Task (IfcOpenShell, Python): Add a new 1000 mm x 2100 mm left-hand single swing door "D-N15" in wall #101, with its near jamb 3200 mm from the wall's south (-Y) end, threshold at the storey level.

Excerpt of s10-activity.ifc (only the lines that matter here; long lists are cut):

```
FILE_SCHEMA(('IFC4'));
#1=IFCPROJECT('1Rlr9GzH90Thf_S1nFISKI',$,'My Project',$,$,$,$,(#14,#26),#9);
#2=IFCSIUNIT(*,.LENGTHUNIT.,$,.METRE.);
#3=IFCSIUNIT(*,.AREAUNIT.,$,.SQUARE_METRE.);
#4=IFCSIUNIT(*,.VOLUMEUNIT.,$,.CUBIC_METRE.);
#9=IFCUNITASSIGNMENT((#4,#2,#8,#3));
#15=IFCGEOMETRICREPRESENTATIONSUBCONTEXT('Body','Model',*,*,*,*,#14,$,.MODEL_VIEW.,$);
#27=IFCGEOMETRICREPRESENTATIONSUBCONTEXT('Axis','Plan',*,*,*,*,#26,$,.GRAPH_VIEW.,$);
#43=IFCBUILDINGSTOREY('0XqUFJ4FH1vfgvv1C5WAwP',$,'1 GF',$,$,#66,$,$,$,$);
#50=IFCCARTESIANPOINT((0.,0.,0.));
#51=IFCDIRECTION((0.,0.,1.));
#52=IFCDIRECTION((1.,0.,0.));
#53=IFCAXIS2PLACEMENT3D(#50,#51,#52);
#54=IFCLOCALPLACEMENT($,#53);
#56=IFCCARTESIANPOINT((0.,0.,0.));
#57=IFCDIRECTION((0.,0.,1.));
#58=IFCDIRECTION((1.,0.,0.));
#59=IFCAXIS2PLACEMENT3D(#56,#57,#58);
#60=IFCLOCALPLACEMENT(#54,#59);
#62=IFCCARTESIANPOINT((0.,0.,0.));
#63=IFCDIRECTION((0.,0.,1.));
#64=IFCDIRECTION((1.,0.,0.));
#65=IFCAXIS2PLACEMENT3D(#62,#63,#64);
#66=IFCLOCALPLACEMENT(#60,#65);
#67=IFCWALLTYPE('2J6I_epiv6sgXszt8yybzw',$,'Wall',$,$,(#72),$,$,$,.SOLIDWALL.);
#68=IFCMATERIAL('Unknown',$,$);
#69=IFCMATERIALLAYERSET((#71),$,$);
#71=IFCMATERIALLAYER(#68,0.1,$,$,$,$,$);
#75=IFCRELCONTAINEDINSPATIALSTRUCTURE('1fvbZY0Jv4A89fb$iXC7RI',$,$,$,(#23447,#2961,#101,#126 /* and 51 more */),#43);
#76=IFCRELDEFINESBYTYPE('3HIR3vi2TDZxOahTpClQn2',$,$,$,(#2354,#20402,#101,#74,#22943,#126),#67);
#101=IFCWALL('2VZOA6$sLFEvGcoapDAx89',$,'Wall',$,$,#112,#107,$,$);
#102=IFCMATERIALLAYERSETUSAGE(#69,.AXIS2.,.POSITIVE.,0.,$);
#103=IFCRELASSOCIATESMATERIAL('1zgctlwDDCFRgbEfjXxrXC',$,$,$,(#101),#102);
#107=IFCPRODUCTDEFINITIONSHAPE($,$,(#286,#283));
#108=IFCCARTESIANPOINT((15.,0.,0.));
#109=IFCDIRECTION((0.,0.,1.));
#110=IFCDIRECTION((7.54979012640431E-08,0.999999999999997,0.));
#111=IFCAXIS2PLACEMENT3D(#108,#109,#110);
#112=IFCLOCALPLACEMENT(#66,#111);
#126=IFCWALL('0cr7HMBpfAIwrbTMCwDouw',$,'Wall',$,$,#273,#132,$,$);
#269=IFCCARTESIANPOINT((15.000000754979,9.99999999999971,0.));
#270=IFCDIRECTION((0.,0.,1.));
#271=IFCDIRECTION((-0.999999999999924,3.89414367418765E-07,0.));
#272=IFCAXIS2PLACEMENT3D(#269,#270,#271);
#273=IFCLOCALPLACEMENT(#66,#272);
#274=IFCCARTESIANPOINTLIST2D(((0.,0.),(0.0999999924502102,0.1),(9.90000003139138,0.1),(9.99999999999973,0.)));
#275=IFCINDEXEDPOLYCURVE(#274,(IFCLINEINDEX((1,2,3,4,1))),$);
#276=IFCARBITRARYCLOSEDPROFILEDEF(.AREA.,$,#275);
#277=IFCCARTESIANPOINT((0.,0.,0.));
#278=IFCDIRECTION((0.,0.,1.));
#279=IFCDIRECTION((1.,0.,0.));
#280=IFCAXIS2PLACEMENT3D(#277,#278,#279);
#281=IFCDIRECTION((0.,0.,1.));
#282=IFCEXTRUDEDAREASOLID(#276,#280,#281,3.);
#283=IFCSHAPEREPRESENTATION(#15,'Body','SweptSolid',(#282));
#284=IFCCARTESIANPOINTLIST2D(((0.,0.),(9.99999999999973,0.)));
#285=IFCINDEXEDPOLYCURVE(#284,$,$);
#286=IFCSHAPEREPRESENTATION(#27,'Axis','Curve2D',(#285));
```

```python
import numpy as np
import ifcopenshell
import ifcopenshell.api.feature
import ifcopenshell.api.geometry
import ifcopenshell.api.root
import ifcopenshell.api.spatial
import ifcopenshell.geom
import ifcopenshell.util.element
import ifcopenshell.util.placement
import ifcopenshell.util.representation
import ifcopenshell.util.shape
import ifcopenshell.util.unit

model = ifcopenshell.open("s10-activity.ifc")
unit_scale = ifcopenshell.util.unit.calculate_unit_scale(model)
settings = ifcopenshell.geom.settings()


def volume(element):
    """Net volume in cubic metres, openings subtracted."""
    shape = ifcopenshell.geom.create_shape(settings, element)
    return ifcopenshell.util.shape.get_volume(shape.geometry)


wall = model.by_guid("2VZOA6$sLFEvGcoapDAx89")
storey = ifcopenshell.util.element.get_container(wall, ifc_class="IfcBuildingStorey")
context = ifcopenshell.util.representation.get_context(model, "Model", "Body", "MODEL_VIEW")
before = volume(wall)

width, height, from_end, sill = 1, 2.1, 3.2, 0.0  # metres

# The wall runs along its own X axis, and the end named is its -X end.
wall_shape = ifcopenshell.geom.create_shape(settings, wall)
x, y, z = ifcopenshell.util.shape.get_vertices(wall_shape.geometry).T
start = x.min() + from_end
face, thickness = float(y.min()), float(y.max() - y.min())
wall_matrix = ifcopenshell.util.placement.get_local_placement(wall.ObjectPlacement)
level = ifcopenshell.util.placement.get_local_placement(storey.ObjectPlacement)[2, 3]


def in_wall(x, y):
    """Placement at x, y metres in the wall's axes, at sill height."""
    matrix = wall_matrix.copy()
    matrix[:, 3] = wall_matrix @ np.array([x / unit_scale, y / unit_scale, 0.0, 1.0])
    matrix[2, 3] = level + sill / unit_scale
    return matrix


# Opening: a box that overshoots both wall faces by 50 mm.
opening = ifcopenshell.api.root.create_entity(model, ifc_class="IfcOpeningElement", predefined_type="OPENING")
box = ifcopenshell.api.geometry.add_wall_representation(
    model, context=context, length=width, height=height, thickness=thickness + 0.1
)
ifcopenshell.api.geometry.assign_representation(model, product=opening, representation=box)
ifcopenshell.api.geometry.edit_object_placement(model, product=opening, matrix=in_wall(start, face - 0.05), is_si=False)
ifcopenshell.api.feature.add_feature(model, feature=opening, element=wall)

door = ifcopenshell.api.root.create_entity(model, ifc_class="IfcDoor", name="D-N15", predefined_type="DOOR")
door.OverallWidth, door.OverallHeight = width / unit_scale, height / unit_scale
door.OperationType = "SINGLE_SWING_LEFT"
body = ifcopenshell.api.geometry.add_door_representation(
    model,
    context=context,
    overall_width=door.OverallWidth,
    overall_height=door.OverallHeight,
    operation_type="SINGLE_SWING_LEFT",
    lining_properties={"LiningDepth": thickness / unit_scale, "ThresholdDepth": thickness / unit_scale},
)
ifcopenshell.api.geometry.assign_representation(model, product=door, representation=body)
ifcopenshell.api.spatial.assign_container(model, products=[door], relating_structure=storey)
ifcopenshell.api.feature.add_filling(model, opening=opening, element=door)

# The lining spans the wall, so the door starts at the wall face.
ifcopenshell.api.geometry.edit_object_placement(model, product=door, matrix=in_wall(start, face), is_si=False)

after = volume(wall)

print(f"wall volume {before:.3f} -> {after:.3f} m3")

model.write("s10-activity-out.ifc")
```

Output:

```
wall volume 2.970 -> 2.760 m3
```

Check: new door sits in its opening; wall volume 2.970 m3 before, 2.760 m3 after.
